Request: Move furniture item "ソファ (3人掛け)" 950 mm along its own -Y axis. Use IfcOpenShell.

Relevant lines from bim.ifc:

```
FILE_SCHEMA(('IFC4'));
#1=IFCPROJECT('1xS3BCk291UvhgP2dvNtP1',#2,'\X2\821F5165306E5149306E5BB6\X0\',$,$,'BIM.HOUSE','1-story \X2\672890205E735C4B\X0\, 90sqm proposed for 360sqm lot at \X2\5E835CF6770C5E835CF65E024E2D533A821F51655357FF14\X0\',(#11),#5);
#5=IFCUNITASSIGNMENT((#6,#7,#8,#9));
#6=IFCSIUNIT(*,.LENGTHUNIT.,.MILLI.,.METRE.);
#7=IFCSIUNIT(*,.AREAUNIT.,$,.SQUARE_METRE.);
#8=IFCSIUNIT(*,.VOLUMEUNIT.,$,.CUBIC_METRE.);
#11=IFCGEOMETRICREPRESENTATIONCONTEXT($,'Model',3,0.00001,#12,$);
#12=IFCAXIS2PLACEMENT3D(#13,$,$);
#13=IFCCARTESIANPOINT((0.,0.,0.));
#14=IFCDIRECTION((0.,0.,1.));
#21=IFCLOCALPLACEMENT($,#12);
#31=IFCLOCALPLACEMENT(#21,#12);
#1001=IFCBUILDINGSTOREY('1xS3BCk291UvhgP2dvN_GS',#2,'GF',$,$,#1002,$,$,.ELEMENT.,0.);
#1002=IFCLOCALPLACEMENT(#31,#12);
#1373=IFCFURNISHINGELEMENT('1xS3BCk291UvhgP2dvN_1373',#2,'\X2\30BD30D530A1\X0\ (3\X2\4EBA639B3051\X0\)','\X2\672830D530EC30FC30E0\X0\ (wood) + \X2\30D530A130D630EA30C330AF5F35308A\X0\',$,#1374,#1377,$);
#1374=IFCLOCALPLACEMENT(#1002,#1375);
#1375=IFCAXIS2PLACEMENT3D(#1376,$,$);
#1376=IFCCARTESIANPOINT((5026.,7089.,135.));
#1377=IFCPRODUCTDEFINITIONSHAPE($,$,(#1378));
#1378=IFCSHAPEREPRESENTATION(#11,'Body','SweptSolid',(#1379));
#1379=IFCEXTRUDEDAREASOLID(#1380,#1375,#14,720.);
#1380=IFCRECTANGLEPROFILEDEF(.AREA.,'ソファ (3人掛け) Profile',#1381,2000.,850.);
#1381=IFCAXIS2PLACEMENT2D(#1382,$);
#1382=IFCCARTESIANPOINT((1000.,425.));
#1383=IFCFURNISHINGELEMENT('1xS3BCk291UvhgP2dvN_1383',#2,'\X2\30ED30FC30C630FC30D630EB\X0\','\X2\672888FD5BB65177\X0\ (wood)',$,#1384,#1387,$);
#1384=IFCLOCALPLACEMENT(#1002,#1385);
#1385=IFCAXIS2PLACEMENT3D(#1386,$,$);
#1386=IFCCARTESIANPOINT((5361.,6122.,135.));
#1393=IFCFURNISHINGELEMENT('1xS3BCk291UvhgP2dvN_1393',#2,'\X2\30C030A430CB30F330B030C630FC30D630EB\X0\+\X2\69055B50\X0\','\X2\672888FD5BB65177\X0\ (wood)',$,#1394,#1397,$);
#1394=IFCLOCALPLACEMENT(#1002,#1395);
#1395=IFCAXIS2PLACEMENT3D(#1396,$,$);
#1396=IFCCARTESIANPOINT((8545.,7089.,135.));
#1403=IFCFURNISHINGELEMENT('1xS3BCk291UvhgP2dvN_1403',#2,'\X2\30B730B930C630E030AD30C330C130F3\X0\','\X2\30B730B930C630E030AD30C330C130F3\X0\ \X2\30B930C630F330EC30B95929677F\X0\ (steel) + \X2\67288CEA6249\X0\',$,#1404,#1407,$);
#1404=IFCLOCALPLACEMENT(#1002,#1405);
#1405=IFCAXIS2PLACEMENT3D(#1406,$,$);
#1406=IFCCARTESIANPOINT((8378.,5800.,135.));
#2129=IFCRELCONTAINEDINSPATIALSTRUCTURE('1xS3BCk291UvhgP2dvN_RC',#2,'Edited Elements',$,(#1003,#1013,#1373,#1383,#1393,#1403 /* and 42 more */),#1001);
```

```python
import ifcopenshell
import ifcopenshell.api.geometry
import ifcopenshell.util.placement
import ifcopenshell.util.unit

model = ifcopenshell.open("bim.ifc")
unit_scale = ifcopenshell.util.unit.calculate_unit_scale(model)

item = model.by_guid("1xS3BCk291UvhgP2dvN_1373")
matrix = ifcopenshell.util.placement.get_local_placement(item.ObjectPlacement)
matrix[:3, 3] -= matrix[:3, 1] * 0.95 / unit_scale
ifcopenshell.api.geometry.edit_object_placement(model, product=item, matrix=matrix, is_si=False)

print(ifcopenshell.util.placement.get_local_placement(item.ObjectPlacement).round(3) + 0.0)

model.write("bim_edited.ifc")
```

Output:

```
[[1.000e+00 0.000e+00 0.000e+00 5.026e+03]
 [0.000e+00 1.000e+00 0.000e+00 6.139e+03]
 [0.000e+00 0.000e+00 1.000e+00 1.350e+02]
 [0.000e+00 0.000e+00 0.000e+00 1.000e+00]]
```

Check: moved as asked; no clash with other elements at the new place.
